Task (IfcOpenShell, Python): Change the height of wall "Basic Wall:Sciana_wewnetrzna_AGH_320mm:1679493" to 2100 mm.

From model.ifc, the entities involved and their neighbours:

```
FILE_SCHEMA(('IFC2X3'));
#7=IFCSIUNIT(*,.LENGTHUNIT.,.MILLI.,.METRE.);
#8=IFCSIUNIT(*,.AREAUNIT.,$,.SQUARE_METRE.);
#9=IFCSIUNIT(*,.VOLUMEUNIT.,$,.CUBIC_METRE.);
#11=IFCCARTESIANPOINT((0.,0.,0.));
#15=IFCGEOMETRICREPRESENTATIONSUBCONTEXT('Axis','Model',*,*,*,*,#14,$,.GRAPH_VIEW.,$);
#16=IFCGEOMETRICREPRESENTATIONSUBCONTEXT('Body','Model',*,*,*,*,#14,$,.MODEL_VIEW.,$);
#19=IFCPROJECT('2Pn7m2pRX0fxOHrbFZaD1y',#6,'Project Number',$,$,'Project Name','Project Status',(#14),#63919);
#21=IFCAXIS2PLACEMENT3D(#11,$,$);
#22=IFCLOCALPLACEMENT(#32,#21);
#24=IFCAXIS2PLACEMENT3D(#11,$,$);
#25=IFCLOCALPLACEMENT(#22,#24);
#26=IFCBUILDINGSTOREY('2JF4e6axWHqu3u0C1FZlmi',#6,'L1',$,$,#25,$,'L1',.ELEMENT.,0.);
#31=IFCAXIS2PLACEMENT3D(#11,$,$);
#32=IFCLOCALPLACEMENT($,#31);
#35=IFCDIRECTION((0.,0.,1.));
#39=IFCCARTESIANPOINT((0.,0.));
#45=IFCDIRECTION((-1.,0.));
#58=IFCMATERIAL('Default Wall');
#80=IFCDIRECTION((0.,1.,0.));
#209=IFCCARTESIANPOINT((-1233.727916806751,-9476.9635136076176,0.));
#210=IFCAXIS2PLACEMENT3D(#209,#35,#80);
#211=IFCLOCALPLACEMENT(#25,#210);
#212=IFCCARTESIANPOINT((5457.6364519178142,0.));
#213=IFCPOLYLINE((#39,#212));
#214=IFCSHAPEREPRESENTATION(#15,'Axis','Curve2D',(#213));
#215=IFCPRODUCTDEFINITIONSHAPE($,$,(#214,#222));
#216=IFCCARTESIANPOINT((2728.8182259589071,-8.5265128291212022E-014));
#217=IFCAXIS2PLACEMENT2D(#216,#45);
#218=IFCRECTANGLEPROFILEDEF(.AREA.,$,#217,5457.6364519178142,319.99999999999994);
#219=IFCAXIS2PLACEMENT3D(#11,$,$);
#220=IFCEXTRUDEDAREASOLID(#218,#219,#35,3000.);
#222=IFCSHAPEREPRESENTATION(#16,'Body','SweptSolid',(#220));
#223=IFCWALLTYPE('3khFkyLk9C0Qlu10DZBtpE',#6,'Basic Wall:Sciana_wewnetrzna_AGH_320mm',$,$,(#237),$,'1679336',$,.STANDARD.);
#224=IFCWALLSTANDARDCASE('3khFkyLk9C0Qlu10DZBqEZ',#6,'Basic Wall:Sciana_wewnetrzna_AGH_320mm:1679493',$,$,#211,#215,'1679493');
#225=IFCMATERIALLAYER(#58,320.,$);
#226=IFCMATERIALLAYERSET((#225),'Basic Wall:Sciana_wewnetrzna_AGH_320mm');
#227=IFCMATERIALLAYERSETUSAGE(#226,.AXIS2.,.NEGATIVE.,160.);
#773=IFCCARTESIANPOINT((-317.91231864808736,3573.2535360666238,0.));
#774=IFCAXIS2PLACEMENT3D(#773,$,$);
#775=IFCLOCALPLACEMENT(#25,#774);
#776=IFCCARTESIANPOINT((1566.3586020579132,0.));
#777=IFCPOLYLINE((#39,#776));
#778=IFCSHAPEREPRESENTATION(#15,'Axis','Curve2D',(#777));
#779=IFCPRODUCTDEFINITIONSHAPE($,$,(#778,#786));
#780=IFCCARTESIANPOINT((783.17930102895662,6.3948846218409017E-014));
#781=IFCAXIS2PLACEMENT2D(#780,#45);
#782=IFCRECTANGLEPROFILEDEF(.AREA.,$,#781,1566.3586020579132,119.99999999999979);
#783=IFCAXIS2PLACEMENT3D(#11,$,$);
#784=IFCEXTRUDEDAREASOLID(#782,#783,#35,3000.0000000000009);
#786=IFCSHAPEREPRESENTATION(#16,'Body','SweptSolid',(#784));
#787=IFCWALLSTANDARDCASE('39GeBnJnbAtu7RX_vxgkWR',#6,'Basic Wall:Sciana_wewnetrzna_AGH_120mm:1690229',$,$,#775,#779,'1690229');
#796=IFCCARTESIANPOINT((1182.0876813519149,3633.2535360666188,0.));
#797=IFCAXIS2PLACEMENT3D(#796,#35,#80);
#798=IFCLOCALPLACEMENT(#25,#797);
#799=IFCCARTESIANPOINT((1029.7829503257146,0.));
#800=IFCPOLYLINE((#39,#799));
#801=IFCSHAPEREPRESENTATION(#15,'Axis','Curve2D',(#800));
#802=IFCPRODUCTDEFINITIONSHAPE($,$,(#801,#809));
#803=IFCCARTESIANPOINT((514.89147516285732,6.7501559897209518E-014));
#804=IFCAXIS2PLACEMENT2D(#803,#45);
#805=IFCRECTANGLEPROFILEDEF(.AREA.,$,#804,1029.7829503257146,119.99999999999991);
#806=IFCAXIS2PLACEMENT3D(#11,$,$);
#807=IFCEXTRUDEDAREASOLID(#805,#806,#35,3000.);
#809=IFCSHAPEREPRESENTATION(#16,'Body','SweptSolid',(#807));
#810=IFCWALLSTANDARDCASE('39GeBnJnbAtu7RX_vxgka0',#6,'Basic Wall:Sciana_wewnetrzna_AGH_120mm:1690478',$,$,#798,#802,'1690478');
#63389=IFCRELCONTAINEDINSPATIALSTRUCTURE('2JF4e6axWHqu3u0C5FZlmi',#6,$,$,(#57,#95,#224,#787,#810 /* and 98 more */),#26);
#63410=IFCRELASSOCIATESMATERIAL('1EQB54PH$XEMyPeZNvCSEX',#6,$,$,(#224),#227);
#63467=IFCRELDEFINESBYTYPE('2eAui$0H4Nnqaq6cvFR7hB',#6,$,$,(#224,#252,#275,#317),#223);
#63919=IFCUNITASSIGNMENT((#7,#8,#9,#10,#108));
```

```python
import ifcopenshell
import ifcopenshell.geom
import ifcopenshell.util.representation
import ifcopenshell.util.shape

model = ifcopenshell.open("model.ifc")
settings = ifcopenshell.geom.settings()


def volume(element):
    """Net volume in cubic metres, openings subtracted."""
    shape = ifcopenshell.geom.create_shape(settings, element)
    return ifcopenshell.util.shape.get_volume(shape.geometry)


wall = model.by_guid("3khFkyLk9C0Qlu10DZBqEZ")
before = volume(wall)

body = ifcopenshell.util.representation.get_representation(wall, "Model", "Body")
solid = body.Items[0]
old_height = solid.Depth
solid.Depth = 2100.0
after = volume(wall)

print(f"height {old_height:g} -> {solid.Depth:g}, volume {before:.3f} -> {after:.3f} m3")

model.write("model_updated.ifc")
```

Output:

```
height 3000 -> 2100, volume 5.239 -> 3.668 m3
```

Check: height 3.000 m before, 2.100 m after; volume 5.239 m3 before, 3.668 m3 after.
